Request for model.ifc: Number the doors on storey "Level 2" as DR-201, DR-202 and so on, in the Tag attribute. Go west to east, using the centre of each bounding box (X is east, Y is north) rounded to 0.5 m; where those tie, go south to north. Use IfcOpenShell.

First a look at what the model holds.

```python
import ifcopenshell
import ifcopenshell.util.element
import ifcopenshell.util.placement

model = ifcopenshell.open("model.ifc")
print(model.schema)
storey = next(s for s in model.by_type("IfcBuildingStorey") if s.Name == "Level 2")
doors = [e for e in ifcopenshell.util.element.get_decomposition(storey) if e.is_a("IfcDoor")]
for e in sorted(doors, key=lambda e: e.id()):
    origin = ifcopenshell.util.placement.get_local_placement(e.ObjectPlacement)[:3, 3]
    print(e.id(), e.Tag, e.Name, origin.round(2) + 0.0, sep=" | ")
```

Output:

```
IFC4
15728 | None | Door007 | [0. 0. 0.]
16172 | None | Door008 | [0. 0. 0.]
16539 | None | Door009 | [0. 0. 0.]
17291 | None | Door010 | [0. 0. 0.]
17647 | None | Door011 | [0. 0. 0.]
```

```python
import ifcopenshell
import ifcopenshell.geom
import ifcopenshell.util.element
import ifcopenshell.util.shape

model = ifcopenshell.open("model.ifc")
settings = ifcopenshell.geom.settings()
settings.set("use-world-coords", True)


def centre(element):
    shape = ifcopenshell.geom.create_shape(settings, element)
    return ifcopenshell.util.shape.get_bbox_centroid(shape.geometry)


storey = next(s for s in model.by_type("IfcBuildingStorey") if s.Name == "Level 2")
doors = [e for e in ifcopenshell.util.element.get_decomposition(storey) if e.is_a("IfcDoor")]

# Insertion points can sit at a corner or the storey origin, so sort by the geometry (in metres).
centres = {e: centre(e) for e in doors}
doors.sort(key=lambda e: (round(centres[e][0] / 0.5), centres[e][1]))

for i, e in enumerate(doors, start=1):
    number = f"DR-2{i:02d}"
    e.Tag = number
    print(e.id(), number)

model.write("model_rev.ifc")
```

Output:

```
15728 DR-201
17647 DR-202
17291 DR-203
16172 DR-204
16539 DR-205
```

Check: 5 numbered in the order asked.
